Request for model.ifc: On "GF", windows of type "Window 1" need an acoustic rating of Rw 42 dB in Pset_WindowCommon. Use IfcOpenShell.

First a look at what the model holds.

```python
import ifcopenshell
import ifcopenshell.util.element

model = ifcopenshell.open("model.ifc")
print(model.schema)
storey = next(s for s in model.by_type("IfcBuildingStorey") if s.Name == "GF")
windows = [e for e in ifcopenshell.util.element.get_decomposition(storey) if e.is_a("IfcWindow")]
seen = {}
for e in windows:
    element_type = ifcopenshell.util.element.get_type(e)
    key = (element_type.Name if element_type != e and element_type else None, ifcopenshell.util.element.get_pset(e, "Pset_WindowCommon", "AcousticRating"))
    seen[key] = seen.get(key, 0) + 1
for (name, value), count in sorted(seen.items(), key=str):
    print(count, "x", name, "|", value)
```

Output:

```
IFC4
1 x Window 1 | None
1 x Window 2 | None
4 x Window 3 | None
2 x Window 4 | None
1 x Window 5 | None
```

```python
import ifcopenshell
import ifcopenshell.api.pset
import ifcopenshell.util.element

model = ifcopenshell.open("model.ifc")

storey = next(s for s in model.by_type("IfcBuildingStorey") if s.Name == "GF")
windows = [e for e in ifcopenshell.util.element.get_decomposition(storey) if e.is_a("IfcWindow")]

count = 0
for e in windows:
    element_type = ifcopenshell.util.element.get_type(e)
    if element_type in (None, e) or element_type.Name != "Window 1":
        continue
    # add_pset returns the element's existing set when there is one.
    pset = ifcopenshell.api.pset.add_pset(model, product=e, name="Pset_WindowCommon")
    ifcopenshell.api.pset.edit_pset(model, pset=pset, properties={"AcousticRating": "Rw 42 dB"})
    count += 1

print(count, "windows updated")

model.write("model_rev.ifc")
```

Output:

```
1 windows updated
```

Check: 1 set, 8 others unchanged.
